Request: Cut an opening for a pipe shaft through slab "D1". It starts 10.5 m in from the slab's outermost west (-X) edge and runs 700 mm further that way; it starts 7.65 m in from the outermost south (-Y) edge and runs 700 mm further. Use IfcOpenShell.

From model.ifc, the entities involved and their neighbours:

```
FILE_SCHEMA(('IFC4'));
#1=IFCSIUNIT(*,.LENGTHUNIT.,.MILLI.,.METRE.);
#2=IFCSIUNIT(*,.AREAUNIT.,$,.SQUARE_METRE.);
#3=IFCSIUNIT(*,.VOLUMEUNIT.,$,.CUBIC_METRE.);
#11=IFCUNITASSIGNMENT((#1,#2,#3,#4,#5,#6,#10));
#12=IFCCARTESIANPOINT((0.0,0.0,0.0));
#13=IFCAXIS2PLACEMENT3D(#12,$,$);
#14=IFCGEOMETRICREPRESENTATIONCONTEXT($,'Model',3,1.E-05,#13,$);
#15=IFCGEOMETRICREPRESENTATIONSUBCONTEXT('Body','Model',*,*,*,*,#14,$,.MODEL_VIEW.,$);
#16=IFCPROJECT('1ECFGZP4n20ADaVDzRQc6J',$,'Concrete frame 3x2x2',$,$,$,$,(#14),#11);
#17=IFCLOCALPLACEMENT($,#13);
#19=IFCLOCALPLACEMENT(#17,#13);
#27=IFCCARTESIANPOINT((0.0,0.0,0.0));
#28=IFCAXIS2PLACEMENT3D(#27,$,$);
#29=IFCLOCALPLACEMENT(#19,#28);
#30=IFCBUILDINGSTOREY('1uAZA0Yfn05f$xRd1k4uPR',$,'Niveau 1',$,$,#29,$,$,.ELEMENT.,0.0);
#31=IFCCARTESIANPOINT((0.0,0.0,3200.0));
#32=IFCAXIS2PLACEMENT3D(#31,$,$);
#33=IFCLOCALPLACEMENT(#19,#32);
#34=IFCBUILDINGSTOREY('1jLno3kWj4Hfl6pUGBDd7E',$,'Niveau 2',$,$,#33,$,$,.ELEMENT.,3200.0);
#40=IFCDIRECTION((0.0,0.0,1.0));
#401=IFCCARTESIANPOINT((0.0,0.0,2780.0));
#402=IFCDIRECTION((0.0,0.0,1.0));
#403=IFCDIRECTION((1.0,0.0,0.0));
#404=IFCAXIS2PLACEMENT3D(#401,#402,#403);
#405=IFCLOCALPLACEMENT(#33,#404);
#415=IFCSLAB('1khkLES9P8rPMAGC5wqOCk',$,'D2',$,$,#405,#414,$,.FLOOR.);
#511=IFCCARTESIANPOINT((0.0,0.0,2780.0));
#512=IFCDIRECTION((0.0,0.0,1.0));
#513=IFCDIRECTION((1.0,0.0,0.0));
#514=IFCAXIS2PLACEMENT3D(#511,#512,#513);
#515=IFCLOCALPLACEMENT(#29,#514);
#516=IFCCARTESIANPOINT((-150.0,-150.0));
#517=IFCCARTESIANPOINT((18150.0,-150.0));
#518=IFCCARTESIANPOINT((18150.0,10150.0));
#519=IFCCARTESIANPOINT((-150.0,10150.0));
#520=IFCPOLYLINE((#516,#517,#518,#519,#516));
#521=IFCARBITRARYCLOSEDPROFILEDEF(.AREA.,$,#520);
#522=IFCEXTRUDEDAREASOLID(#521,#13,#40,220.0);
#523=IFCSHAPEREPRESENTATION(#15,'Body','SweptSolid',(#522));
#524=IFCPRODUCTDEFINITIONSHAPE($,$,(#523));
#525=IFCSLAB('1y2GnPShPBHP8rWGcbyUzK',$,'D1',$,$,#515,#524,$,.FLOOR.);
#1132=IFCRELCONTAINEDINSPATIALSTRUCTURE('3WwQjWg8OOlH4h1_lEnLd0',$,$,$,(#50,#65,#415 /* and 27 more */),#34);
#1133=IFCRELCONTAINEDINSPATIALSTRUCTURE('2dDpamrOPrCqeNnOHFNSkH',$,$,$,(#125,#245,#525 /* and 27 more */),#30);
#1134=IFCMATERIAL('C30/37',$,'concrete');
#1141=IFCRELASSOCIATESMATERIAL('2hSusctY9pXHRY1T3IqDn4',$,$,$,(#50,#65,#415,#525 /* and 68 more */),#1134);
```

```python
import numpy as np
import ifcopenshell
import ifcopenshell.api.feature
import ifcopenshell.api.geometry
import ifcopenshell.api.root
import ifcopenshell.geom
import ifcopenshell.util.placement
import ifcopenshell.util.representation
import ifcopenshell.util.shape
import ifcopenshell.util.unit

model = ifcopenshell.open("model.ifc")
unit_scale = ifcopenshell.util.unit.calculate_unit_scale(model)
settings = ifcopenshell.geom.settings()


def volume(element):
    """Net volume in cubic metres, openings subtracted."""
    shape = ifcopenshell.geom.create_shape(settings, element)
    return ifcopenshell.util.shape.get_volume(shape.geometry)


slab = model.by_guid("1y2GnPShPBHP8rWGcbyUzK")
before = volume(slab)

# Extent in the slab's own axes, in metres. The edges named are its -X and -Y sides.
slab_shape = ifcopenshell.geom.create_shape(settings, slab)
vertices = ifcopenshell.util.shape.get_vertices(slab_shape.geometry)
x_min, y_min, bottom = vertices.min(axis=0)
top = vertices[:, 2].max()

opening = ifcopenshell.api.root.create_entity(model, ifc_class="IfcOpeningElement", name="Pipe shaft opening", predefined_type="OPENING")
context = ifcopenshell.util.representation.get_context(model, "Model", "Body", "MODEL_VIEW")
width, depth = 0.7, 0.7
outline = [(0.0, 0.0), (width, 0.0), (width, depth), (0.0, depth), (0.0, 0.0)]
# Overshoot both faces by 50 mm so the cut is clean.
shape = ifcopenshell.api.geometry.add_slab_representation(
    model, context=context, depth=top - bottom + 0.1, polyline=outline
)
ifcopenshell.api.geometry.assign_representation(model, product=opening, representation=shape)

matrix = ifcopenshell.util.placement.get_local_placement(slab.ObjectPlacement)
matrix[:, 3] = matrix @ np.append(np.array([x_min + 10.5, y_min + 7.65, bottom - 0.05]) / unit_scale, 1.0)
ifcopenshell.api.geometry.edit_object_placement(model, product=opening, matrix=matrix, is_si=False)
ifcopenshell.api.feature.add_feature(model, feature=opening, element=slab)

after = volume(slab)

print(f"slab volume {before:.3f} -> {after:.3f} m3")

model.write("model-out.ifc")
```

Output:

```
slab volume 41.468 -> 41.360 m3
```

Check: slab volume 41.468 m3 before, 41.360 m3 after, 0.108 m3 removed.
